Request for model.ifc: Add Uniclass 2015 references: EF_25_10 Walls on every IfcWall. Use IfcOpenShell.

First a look at what the model holds.

```python
import ifcopenshell

model = ifcopenshell.open("model.ifc")
print(model.schema)
print("classifications:", [c.Name for c in model.by_type("IfcClassification")])
for ifc_class in ("IfcDoor", "IfcRoof", "IfcStair", "IfcWall", "IfcWindow"):
    print(ifc_class, len(model.by_type(ifc_class)))
```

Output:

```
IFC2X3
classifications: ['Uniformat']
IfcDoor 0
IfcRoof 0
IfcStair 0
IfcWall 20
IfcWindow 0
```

```python
import ifcopenshell
import ifcopenshell.api.classification

model = ifcopenshell.open("model.ifc")

# IFC2X3 requires Source and Edition and has no link from the project to the system.
system = model.create_entity("IfcClassification", Source="NBS", Edition="2015", Name="Uniclass 2015")

codes = {
    "IfcWall": ("EF_25_10", "Walls"),
}
for ifc_class, (code, name) in codes.items():
    products = model.by_type(ifc_class)
    ifcopenshell.api.classification.add_reference(
        model, products=products, classification=system, identification=code, name=name
    )
    print(code, len(products))

model.write("model-out.ifc")
```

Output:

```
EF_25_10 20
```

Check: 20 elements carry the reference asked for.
